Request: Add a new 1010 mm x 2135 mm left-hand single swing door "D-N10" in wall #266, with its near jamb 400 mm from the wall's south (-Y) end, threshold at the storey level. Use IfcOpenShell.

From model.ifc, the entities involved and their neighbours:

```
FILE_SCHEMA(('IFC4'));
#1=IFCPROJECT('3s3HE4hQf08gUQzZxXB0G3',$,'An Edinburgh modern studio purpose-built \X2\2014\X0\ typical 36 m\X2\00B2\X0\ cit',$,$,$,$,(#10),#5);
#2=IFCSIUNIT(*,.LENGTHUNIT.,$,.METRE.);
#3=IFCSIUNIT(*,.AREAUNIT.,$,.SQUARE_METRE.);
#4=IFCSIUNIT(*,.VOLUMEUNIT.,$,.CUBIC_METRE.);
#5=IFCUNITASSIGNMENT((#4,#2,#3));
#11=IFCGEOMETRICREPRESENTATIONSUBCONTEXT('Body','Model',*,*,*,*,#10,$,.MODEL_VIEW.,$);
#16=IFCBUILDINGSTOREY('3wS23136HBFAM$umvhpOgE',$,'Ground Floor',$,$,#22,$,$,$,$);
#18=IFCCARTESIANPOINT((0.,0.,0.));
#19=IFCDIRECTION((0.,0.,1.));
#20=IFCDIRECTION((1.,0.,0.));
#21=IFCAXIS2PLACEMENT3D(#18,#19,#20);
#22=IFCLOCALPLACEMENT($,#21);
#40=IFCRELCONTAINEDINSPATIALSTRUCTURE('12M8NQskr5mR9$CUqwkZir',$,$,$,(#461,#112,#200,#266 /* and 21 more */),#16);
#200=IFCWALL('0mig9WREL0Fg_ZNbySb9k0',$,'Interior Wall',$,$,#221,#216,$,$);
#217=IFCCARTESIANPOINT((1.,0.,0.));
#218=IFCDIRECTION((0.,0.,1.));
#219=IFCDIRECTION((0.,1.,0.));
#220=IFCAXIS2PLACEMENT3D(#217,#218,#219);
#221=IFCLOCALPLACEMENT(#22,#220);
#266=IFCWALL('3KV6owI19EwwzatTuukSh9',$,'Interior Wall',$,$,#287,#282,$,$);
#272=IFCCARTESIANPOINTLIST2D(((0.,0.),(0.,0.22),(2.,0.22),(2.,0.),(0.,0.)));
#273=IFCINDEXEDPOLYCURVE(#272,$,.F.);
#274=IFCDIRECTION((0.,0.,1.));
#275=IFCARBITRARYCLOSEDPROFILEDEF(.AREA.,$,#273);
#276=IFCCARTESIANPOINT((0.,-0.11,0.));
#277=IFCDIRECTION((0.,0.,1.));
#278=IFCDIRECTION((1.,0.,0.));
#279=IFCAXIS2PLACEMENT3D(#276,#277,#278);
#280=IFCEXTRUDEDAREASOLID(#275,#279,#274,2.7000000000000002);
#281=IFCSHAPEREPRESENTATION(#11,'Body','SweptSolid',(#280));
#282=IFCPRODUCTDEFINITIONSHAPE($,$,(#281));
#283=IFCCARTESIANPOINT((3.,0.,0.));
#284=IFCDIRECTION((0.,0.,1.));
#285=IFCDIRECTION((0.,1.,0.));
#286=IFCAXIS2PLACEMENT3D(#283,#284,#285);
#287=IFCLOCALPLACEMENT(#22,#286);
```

```python
import numpy as np
import ifcopenshell
import ifcopenshell.api.feature
import ifcopenshell.api.geometry
import ifcopenshell.api.root
import ifcopenshell.api.spatial
import ifcopenshell.geom
import ifcopenshell.util.element
import ifcopenshell.util.placement
import ifcopenshell.util.representation
import ifcopenshell.util.shape
import ifcopenshell.util.unit

model = ifcopenshell.open("model.ifc")
unit_scale = ifcopenshell.util.unit.calculate_unit_scale(model)
settings = ifcopenshell.geom.settings()


def volume(element):
    """Net volume in cubic metres, openings subtracted."""
    shape = ifcopenshell.geom.create_shape(settings, element)
    return ifcopenshell.util.shape.get_volume(shape.geometry)


wall = model.by_guid("3KV6owI19EwwzatTuukSh9")
storey = ifcopenshell.util.element.get_container(wall, ifc_class="IfcBuildingStorey")
context = ifcopenshell.util.representation.get_context(model, "Model", "Body", "MODEL_VIEW")
before = volume(wall)

width, height, from_end, sill = 1.01, 2.135, 0.4, 0.0  # metres

# The wall runs along its own X axis, and the end named is its -X end.
wall_shape = ifcopenshell.geom.create_shape(settings, wall)
x, y, z = ifcopenshell.util.shape.get_vertices(wall_shape.geometry).T
start = x.min() + from_end
face, thickness = float(y.min()), float(y.max() - y.min())
wall_matrix = ifcopenshell.util.placement.get_local_placement(wall.ObjectPlacement)
level = ifcopenshell.util.placement.get_local_placement(storey.ObjectPlacement)[2, 3]


def in_wall(x, y):
    """Placement at x, y metres in the wall's axes, at sill height."""
    matrix = wall_matrix.copy()
    matrix[:, 3] = wall_matrix @ np.array([x / unit_scale, y / unit_scale, 0.0, 1.0])
    matrix[2, 3] = level + sill / unit_scale
    return matrix


# Opening: a box that overshoots both wall faces by 50 mm.
opening = ifcopenshell.api.root.create_entity(model, ifc_class="IfcOpeningElement", predefined_type="OPENING")
box = ifcopenshell.api.geometry.add_wall_representation(
    model, context=context, length=width, height=height, thickness=thickness + 0.1
)
ifcopenshell.api.geometry.assign_representation(model, product=opening, representation=box)
ifcopenshell.api.geometry.edit_object_placement(model, product=opening, matrix=in_wall(start, face - 0.05), is_si=False)
ifcopenshell.api.feature.add_feature(model, feature=opening, element=wall)

door = ifcopenshell.api.root.create_entity(model, ifc_class="IfcDoor", name="D-N10", predefined_type="DOOR")
door.OverallWidth, door.OverallHeight = width / unit_scale, height / unit_scale
door.OperationType = "SINGLE_SWING_LEFT"
body = ifcopenshell.api.geometry.add_door_representation(
    model,
    context=context,
    overall_width=door.OverallWidth,
    overall_height=door.OverallHeight,
    operation_type="SINGLE_SWING_LEFT",
    lining_properties={"LiningDepth": thickness / unit_scale, "ThresholdDepth": thickness / unit_scale},
)
ifcopenshell.api.geometry.assign_representation(model, product=door, representation=body)
ifcopenshell.api.spatial.assign_container(model, products=[door], relating_structure=storey)
ifcopenshell.api.feature.add_filling(model, opening=opening, element=door)

# The lining spans the wall, so the door starts at the wall face.
ifcopenshell.api.geometry.edit_object_placement(model, product=door, matrix=in_wall(start, face), is_si=False)

after = volume(wall)

print(f"wall volume {before:.3f} -> {after:.3f} m3")

model.write("model_v2.ifc")
```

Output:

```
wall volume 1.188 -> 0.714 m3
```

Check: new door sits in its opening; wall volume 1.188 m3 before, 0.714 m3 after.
